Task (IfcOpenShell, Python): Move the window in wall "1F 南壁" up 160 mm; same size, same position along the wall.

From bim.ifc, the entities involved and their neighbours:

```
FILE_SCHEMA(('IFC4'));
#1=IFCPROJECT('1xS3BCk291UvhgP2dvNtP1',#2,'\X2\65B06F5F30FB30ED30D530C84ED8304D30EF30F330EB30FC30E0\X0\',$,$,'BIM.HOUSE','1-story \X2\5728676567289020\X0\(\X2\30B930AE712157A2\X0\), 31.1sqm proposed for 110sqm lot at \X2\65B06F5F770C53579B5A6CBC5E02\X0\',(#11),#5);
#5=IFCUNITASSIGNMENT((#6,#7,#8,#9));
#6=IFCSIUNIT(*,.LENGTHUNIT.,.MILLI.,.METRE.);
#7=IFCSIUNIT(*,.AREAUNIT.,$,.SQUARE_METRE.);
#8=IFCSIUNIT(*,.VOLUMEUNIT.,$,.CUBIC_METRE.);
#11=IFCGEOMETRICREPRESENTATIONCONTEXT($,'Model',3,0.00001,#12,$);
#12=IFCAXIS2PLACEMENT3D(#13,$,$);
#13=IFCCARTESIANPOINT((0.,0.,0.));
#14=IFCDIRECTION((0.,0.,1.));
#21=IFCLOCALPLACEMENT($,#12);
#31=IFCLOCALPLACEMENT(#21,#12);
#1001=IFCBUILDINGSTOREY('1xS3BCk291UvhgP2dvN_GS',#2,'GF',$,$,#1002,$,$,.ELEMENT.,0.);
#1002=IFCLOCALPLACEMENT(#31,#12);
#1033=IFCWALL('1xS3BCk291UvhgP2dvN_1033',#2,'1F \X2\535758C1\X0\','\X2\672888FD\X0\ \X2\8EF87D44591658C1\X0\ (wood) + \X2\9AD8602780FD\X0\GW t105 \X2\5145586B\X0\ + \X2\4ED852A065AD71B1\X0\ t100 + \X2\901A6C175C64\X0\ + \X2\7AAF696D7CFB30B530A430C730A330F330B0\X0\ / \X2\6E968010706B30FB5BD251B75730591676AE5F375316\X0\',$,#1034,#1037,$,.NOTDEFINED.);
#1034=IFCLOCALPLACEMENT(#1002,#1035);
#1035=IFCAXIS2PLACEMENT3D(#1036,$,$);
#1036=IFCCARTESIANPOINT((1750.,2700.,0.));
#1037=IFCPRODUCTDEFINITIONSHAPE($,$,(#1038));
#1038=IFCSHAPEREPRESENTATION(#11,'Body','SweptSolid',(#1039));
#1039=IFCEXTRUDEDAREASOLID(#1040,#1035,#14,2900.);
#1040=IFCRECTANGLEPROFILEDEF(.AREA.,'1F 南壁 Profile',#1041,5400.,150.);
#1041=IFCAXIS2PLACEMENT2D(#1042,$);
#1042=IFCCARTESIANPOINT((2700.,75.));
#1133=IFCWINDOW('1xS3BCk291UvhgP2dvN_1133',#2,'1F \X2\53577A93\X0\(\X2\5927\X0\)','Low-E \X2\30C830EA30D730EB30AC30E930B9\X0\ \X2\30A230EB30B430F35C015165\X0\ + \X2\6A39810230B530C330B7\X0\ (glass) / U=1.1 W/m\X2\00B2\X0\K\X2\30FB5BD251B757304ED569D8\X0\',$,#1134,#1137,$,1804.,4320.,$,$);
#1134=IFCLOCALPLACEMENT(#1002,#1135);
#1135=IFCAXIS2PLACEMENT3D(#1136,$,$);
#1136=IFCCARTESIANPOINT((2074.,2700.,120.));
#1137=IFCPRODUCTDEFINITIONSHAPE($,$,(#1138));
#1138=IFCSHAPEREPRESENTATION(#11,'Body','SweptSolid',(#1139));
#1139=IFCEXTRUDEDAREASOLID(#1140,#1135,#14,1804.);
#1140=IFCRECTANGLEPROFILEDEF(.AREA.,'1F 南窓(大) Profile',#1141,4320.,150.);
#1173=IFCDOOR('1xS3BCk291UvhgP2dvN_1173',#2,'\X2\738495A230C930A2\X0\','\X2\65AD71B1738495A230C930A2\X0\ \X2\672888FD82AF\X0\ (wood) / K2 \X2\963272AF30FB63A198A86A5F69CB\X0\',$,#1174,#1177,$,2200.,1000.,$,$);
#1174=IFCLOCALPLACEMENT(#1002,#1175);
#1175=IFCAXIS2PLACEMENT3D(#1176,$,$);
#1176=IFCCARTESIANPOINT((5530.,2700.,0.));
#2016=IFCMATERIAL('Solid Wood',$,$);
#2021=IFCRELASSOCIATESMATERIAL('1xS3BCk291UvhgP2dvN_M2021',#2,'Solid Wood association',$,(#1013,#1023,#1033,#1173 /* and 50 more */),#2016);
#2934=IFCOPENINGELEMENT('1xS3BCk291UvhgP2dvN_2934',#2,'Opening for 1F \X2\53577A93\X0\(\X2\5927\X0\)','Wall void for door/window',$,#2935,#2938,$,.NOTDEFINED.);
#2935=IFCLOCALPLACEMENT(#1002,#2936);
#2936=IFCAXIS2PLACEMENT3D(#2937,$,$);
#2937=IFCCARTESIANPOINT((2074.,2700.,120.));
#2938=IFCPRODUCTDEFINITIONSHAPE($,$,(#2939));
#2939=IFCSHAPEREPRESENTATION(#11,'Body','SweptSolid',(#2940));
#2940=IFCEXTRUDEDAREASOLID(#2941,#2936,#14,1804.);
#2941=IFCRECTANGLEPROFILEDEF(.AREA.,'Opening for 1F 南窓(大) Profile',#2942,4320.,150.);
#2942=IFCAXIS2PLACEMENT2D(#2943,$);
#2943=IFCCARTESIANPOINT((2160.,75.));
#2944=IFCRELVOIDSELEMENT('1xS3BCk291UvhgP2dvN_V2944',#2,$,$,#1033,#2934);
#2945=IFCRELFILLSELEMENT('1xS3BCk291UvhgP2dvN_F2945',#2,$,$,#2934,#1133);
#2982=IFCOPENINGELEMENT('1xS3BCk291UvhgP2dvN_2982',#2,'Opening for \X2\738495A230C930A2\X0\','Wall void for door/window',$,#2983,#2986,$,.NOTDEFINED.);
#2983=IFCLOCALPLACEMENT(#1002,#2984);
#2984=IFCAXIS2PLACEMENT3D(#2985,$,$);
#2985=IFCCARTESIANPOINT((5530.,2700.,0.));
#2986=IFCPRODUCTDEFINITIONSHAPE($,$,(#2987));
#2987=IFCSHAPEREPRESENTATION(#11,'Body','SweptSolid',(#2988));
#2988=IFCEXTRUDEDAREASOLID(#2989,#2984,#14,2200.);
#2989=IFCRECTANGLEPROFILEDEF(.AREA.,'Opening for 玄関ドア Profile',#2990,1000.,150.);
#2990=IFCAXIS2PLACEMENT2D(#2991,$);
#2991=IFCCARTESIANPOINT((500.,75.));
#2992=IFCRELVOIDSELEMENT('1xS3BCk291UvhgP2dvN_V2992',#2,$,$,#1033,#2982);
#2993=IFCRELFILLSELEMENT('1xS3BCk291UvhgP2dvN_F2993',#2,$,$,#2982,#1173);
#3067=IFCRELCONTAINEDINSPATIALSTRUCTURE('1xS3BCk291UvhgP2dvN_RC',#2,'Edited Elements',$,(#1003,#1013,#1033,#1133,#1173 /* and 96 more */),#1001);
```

```python
import numpy as np
import ifcopenshell
import ifcopenshell.api.geometry
import ifcopenshell.util.placement
import ifcopenshell.util.unit

model = ifcopenshell.open("bim.ifc")
unit_scale = ifcopenshell.util.unit.calculate_unit_scale(model)

window = model.by_guid("1xS3BCk291UvhgP2dvN_1133")
opening = window.FillsVoids[0].RelatingOpeningElement
dz = 160.0

shift = np.array([0.0, 0.0, dz])
# The window is not placed relative to its opening, so move both.
for product in (opening, window):
    matrix = ifcopenshell.util.placement.get_local_placement(product.ObjectPlacement)
    matrix[:3, 3] += shift
    ifcopenshell.api.geometry.edit_object_placement(model, product=product, matrix=matrix, is_si=False)

print(f"moved by {dz * unit_scale:+.3f} m")

model.write("bim_updated.ifc")
```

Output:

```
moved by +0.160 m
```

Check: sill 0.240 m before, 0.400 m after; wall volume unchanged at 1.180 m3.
